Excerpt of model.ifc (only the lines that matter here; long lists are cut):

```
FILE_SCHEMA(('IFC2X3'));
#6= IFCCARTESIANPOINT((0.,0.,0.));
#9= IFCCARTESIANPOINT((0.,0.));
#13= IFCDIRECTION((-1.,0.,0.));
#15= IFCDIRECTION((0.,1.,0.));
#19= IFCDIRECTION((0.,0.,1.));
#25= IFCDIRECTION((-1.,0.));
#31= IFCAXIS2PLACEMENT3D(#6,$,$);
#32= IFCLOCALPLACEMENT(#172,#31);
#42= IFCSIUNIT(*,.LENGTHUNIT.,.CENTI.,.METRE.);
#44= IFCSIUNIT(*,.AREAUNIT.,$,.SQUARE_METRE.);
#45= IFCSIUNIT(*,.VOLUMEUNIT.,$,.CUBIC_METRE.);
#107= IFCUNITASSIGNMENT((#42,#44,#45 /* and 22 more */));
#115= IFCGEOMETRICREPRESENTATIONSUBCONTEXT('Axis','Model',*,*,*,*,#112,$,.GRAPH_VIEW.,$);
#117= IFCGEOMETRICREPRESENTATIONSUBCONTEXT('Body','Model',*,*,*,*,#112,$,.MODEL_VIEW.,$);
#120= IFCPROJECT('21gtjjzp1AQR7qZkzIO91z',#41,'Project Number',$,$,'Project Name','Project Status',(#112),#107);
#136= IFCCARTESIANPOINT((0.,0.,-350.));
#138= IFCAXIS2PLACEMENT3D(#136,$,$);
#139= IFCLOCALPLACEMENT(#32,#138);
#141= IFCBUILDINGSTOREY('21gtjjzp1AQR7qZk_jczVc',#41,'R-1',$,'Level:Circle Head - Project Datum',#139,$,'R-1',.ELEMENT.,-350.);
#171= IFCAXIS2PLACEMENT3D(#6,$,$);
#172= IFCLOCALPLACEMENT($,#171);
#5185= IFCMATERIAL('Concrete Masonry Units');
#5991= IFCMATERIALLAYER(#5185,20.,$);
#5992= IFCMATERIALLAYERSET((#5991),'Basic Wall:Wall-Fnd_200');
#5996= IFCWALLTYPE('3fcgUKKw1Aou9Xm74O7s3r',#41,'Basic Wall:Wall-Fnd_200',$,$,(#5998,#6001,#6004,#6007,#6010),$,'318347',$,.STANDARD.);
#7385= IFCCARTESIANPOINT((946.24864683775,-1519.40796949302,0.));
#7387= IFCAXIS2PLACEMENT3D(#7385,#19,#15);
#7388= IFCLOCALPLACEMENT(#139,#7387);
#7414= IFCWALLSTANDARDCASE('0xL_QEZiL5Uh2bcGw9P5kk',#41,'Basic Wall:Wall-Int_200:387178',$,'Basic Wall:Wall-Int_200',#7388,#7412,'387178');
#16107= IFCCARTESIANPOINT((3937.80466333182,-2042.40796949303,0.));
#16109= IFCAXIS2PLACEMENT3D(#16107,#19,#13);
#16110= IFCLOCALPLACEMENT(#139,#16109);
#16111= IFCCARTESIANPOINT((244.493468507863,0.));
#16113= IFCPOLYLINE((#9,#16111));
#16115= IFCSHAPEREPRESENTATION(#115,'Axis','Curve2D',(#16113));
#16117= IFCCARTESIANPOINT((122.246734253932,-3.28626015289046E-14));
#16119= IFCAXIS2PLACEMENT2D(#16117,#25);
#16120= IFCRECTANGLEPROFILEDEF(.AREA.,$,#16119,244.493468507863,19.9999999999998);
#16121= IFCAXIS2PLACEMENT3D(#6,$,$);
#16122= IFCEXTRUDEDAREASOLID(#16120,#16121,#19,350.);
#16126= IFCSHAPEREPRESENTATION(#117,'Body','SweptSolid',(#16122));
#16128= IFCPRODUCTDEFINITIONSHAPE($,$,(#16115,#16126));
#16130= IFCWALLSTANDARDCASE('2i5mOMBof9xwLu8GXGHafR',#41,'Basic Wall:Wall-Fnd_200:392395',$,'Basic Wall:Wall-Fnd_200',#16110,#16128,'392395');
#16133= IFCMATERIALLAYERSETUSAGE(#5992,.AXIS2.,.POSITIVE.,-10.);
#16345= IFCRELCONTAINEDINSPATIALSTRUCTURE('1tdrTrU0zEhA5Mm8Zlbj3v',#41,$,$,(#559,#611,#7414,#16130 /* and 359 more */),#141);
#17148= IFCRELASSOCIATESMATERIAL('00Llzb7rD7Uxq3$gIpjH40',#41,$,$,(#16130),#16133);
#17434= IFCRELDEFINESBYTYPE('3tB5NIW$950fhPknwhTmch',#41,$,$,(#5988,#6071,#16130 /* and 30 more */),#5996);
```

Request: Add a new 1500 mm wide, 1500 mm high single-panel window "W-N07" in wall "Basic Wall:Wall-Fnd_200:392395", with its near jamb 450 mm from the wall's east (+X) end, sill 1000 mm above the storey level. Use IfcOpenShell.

```python
import numpy as np
import ifcopenshell
import ifcopenshell.api.feature
import ifcopenshell.api.geometry
import ifcopenshell.api.root
import ifcopenshell.api.spatial
import ifcopenshell.api.type
import ifcopenshell.geom
import ifcopenshell.util.element
import ifcopenshell.util.placement
import ifcopenshell.util.representation
import ifcopenshell.util.shape
import ifcopenshell.util.unit

model = ifcopenshell.open("model.ifc")
unit_scale = ifcopenshell.util.unit.calculate_unit_scale(model)
settings = ifcopenshell.geom.settings()


def volume(element):
    """Net volume in cubic metres, openings subtracted."""
    shape = ifcopenshell.geom.create_shape(settings, element)
    return ifcopenshell.util.shape.get_volume(shape.geometry)


wall = model.by_id(16130)
storey = ifcopenshell.util.element.get_container(wall, ifc_class="IfcBuildingStorey")
context = ifcopenshell.util.representation.get_context(model, "Model", "Body", "MODEL_VIEW")
before = volume(wall)

width, height, from_end, sill = 1.5, 1.5, 0.45, 1  # metres

# The wall runs along its own X axis, and the end named is its -X end.
wall_shape = ifcopenshell.geom.create_shape(settings, wall)
x, y, z = ifcopenshell.util.shape.get_vertices(wall_shape.geometry).T
start = x.min() + from_end
face, thickness = float(y.min()), float(y.max() - y.min())
wall_matrix = ifcopenshell.util.placement.get_local_placement(wall.ObjectPlacement)
level = ifcopenshell.util.placement.get_local_placement(storey.ObjectPlacement)[2, 3]


def in_wall(x, y):
    """Placement at x, y metres in the wall's axes, at sill height."""
    matrix = wall_matrix.copy()
    matrix[:, 3] = wall_matrix @ np.array([x / unit_scale, y / unit_scale, 0.0, 1.0])
    matrix[2, 3] = level + sill / unit_scale
    return matrix


# Opening: a box that overshoots both wall faces by 50 mm.
opening = ifcopenshell.api.root.create_entity(model, ifc_class="IfcOpeningElement")
box = ifcopenshell.api.geometry.add_wall_representation(
    model, context=context, length=width, height=height, thickness=thickness + 0.1
)
ifcopenshell.api.geometry.assign_representation(model, product=opening, representation=box)
ifcopenshell.api.geometry.edit_object_placement(model, product=opening, matrix=in_wall(start, face - 0.05), is_si=False)
ifcopenshell.api.feature.add_feature(model, feature=opening, element=wall)

window = ifcopenshell.api.root.create_entity(model, ifc_class="IfcWindow", name="W-N07")
window.OverallWidth, window.OverallHeight = width / unit_scale, height / unit_scale
body = ifcopenshell.api.geometry.add_window_representation(
    model,
    context=context,
    overall_width=window.OverallWidth,
    overall_height=window.OverallHeight,
    partition_type="SINGLE_PANEL",
)
ifcopenshell.api.geometry.assign_representation(model, product=window, representation=body)
ifcopenshell.api.spatial.assign_container(model, products=[window], relating_structure=storey)
fills = ifcopenshell.api.feature.add_filling(model, opening=opening, element=window)
fills.OwnerHistory = window.OwnerHistory  # required in IFC2X3

# IFC2X3 keeps the operation on the window style.
style = ifcopenshell.api.root.create_entity(model, ifc_class="IfcWindowStyle", name="W-N07")
style.OperationType, style.ConstructionType = "SINGLE_PANEL", "NOTDEFINED"
style.ParameterTakesPrecedence = style.Sizeable = False
ifcopenshell.api.type.assign_type(model, related_objects=[window], relating_type=style)

# Centre the window in the wall's thickness.
ifcopenshell.api.geometry.edit_object_placement(model, product=window, matrix=in_wall(start, face), is_si=False)
window_shape = ifcopenshell.geom.create_shape(settings, window)
depth = ifcopenshell.util.shape.get_vertices(window_shape.geometry)[:, 1]
offset = face + thickness / 2 - (depth.min() + depth.max()) / 2
ifcopenshell.api.geometry.edit_object_placement(model, product=window, matrix=in_wall(start, offset), is_si=False)

after = volume(wall)

print(f"wall volume {before:.3f} -> {after:.3f} m3")

model.write("model_v2.ifc")
```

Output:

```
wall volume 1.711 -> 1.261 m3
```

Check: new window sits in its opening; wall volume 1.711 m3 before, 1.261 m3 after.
